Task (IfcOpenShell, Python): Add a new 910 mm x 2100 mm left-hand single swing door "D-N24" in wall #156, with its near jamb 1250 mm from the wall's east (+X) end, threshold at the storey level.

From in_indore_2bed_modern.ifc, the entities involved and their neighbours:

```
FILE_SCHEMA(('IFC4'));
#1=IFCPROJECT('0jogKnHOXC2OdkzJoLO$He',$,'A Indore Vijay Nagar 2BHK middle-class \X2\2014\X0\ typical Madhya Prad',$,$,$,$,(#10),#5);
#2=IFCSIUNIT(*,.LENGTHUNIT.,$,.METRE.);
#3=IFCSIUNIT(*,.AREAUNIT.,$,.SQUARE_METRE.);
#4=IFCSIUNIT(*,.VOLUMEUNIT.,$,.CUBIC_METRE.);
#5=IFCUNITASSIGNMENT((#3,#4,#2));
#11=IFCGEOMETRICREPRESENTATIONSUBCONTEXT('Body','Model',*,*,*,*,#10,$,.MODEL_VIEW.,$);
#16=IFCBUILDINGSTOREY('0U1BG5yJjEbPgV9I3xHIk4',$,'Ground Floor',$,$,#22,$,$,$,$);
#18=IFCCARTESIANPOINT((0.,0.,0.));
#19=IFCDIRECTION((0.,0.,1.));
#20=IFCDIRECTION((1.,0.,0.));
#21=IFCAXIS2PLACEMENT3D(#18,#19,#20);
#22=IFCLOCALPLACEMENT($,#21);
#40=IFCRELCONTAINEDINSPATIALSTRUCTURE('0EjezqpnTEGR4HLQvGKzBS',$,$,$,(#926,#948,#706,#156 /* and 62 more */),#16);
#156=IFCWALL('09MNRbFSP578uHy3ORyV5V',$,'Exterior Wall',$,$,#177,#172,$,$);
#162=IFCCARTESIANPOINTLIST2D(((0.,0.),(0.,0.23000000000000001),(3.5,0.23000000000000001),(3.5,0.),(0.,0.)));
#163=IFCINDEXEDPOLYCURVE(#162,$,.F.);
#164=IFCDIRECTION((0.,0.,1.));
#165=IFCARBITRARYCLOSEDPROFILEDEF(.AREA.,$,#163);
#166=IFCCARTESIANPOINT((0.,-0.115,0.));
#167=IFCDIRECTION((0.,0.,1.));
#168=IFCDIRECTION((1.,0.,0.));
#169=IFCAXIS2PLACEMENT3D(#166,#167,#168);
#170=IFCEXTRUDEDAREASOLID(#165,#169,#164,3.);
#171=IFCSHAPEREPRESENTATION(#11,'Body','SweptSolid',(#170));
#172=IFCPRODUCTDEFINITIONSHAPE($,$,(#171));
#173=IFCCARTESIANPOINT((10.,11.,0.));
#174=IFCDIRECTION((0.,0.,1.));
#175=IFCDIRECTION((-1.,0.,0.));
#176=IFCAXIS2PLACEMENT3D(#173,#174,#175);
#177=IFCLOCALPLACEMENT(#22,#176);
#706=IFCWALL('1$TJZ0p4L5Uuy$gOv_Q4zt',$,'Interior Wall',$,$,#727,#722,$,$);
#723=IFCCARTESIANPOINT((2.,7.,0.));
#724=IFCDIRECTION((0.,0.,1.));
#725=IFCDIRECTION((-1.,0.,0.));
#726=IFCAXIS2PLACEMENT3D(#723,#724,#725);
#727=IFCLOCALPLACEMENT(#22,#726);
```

```python
import numpy as np
import ifcopenshell
import ifcopenshell.api.feature
import ifcopenshell.api.geometry
import ifcopenshell.api.root
import ifcopenshell.api.spatial
import ifcopenshell.geom
import ifcopenshell.util.element
import ifcopenshell.util.placement
import ifcopenshell.util.representation
import ifcopenshell.util.shape
import ifcopenshell.util.unit

model = ifcopenshell.open("in_indore_2bed_modern.ifc")
unit_scale = ifcopenshell.util.unit.calculate_unit_scale(model)
settings = ifcopenshell.geom.settings()


def volume(element):
    """Net volume in cubic metres, openings subtracted."""
    shape = ifcopenshell.geom.create_shape(settings, element)
    return ifcopenshell.util.shape.get_volume(shape.geometry)


wall = model.by_id(156)
storey = ifcopenshell.util.element.get_container(wall, ifc_class="IfcBuildingStorey")
context = ifcopenshell.util.representation.get_context(model, "Model", "Body", "MODEL_VIEW")
before = volume(wall)

width, height, from_end, sill = 0.91, 2.1, 1.25, 0.0  # metres

# The wall runs along its own X axis, and the end named is its -X end.
wall_shape = ifcopenshell.geom.create_shape(settings, wall)
x, y, z = ifcopenshell.util.shape.get_vertices(wall_shape.geometry).T
start = x.min() + from_end
face, thickness = float(y.min()), float(y.max() - y.min())
wall_matrix = ifcopenshell.util.placement.get_local_placement(wall.ObjectPlacement)
level = ifcopenshell.util.placement.get_local_placement(storey.ObjectPlacement)[2, 3]


def in_wall(x, y):
    """Placement at x, y metres in the wall's axes, at sill height."""
    matrix = wall_matrix.copy()
    matrix[:, 3] = wall_matrix @ np.array([x / unit_scale, y / unit_scale, 0.0, 1.0])
    matrix[2, 3] = level + sill / unit_scale
    return matrix


# Opening: a box that overshoots both wall faces by 50 mm.
opening = ifcopenshell.api.root.create_entity(model, ifc_class="IfcOpeningElement", predefined_type="OPENING")
box = ifcopenshell.api.geometry.add_wall_representation(
    model, context=context, length=width, height=height, thickness=thickness + 0.1
)
ifcopenshell.api.geometry.assign_representation(model, product=opening, representation=box)
ifcopenshell.api.geometry.edit_object_placement(model, product=opening, matrix=in_wall(start, face - 0.05), is_si=False)
ifcopenshell.api.feature.add_feature(model, feature=opening, element=wall)

door = ifcopenshell.api.root.create_entity(model, ifc_class="IfcDoor", name="D-N24", predefined_type="DOOR")
door.OverallWidth, door.OverallHeight = width / unit_scale, height / unit_scale
door.OperationType = "SINGLE_SWING_LEFT"
body = ifcopenshell.api.geometry.add_door_representation(
    model,
    context=context,
    overall_width=door.OverallWidth,
    overall_height=door.OverallHeight,
    operation_type="SINGLE_SWING_LEFT",
    lining_properties={"LiningDepth": thickness / unit_scale, "ThresholdDepth": thickness / unit_scale},
)
ifcopenshell.api.geometry.assign_representation(model, product=door, representation=body)
ifcopenshell.api.spatial.assign_container(model, products=[door], relating_structure=storey)
ifcopenshell.api.feature.add_filling(model, opening=opening, element=door)

# The lining spans the wall, so the door starts at the wall face.
ifcopenshell.api.geometry.edit_object_placement(model, product=door, matrix=in_wall(start, face), is_si=False)

after = volume(wall)

print(f"wall volume {before:.3f} -> {after:.3f} m3")

model.write("in_indore_2bed_modern_v2.ifc")
```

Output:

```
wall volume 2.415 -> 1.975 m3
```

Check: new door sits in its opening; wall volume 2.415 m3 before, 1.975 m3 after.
